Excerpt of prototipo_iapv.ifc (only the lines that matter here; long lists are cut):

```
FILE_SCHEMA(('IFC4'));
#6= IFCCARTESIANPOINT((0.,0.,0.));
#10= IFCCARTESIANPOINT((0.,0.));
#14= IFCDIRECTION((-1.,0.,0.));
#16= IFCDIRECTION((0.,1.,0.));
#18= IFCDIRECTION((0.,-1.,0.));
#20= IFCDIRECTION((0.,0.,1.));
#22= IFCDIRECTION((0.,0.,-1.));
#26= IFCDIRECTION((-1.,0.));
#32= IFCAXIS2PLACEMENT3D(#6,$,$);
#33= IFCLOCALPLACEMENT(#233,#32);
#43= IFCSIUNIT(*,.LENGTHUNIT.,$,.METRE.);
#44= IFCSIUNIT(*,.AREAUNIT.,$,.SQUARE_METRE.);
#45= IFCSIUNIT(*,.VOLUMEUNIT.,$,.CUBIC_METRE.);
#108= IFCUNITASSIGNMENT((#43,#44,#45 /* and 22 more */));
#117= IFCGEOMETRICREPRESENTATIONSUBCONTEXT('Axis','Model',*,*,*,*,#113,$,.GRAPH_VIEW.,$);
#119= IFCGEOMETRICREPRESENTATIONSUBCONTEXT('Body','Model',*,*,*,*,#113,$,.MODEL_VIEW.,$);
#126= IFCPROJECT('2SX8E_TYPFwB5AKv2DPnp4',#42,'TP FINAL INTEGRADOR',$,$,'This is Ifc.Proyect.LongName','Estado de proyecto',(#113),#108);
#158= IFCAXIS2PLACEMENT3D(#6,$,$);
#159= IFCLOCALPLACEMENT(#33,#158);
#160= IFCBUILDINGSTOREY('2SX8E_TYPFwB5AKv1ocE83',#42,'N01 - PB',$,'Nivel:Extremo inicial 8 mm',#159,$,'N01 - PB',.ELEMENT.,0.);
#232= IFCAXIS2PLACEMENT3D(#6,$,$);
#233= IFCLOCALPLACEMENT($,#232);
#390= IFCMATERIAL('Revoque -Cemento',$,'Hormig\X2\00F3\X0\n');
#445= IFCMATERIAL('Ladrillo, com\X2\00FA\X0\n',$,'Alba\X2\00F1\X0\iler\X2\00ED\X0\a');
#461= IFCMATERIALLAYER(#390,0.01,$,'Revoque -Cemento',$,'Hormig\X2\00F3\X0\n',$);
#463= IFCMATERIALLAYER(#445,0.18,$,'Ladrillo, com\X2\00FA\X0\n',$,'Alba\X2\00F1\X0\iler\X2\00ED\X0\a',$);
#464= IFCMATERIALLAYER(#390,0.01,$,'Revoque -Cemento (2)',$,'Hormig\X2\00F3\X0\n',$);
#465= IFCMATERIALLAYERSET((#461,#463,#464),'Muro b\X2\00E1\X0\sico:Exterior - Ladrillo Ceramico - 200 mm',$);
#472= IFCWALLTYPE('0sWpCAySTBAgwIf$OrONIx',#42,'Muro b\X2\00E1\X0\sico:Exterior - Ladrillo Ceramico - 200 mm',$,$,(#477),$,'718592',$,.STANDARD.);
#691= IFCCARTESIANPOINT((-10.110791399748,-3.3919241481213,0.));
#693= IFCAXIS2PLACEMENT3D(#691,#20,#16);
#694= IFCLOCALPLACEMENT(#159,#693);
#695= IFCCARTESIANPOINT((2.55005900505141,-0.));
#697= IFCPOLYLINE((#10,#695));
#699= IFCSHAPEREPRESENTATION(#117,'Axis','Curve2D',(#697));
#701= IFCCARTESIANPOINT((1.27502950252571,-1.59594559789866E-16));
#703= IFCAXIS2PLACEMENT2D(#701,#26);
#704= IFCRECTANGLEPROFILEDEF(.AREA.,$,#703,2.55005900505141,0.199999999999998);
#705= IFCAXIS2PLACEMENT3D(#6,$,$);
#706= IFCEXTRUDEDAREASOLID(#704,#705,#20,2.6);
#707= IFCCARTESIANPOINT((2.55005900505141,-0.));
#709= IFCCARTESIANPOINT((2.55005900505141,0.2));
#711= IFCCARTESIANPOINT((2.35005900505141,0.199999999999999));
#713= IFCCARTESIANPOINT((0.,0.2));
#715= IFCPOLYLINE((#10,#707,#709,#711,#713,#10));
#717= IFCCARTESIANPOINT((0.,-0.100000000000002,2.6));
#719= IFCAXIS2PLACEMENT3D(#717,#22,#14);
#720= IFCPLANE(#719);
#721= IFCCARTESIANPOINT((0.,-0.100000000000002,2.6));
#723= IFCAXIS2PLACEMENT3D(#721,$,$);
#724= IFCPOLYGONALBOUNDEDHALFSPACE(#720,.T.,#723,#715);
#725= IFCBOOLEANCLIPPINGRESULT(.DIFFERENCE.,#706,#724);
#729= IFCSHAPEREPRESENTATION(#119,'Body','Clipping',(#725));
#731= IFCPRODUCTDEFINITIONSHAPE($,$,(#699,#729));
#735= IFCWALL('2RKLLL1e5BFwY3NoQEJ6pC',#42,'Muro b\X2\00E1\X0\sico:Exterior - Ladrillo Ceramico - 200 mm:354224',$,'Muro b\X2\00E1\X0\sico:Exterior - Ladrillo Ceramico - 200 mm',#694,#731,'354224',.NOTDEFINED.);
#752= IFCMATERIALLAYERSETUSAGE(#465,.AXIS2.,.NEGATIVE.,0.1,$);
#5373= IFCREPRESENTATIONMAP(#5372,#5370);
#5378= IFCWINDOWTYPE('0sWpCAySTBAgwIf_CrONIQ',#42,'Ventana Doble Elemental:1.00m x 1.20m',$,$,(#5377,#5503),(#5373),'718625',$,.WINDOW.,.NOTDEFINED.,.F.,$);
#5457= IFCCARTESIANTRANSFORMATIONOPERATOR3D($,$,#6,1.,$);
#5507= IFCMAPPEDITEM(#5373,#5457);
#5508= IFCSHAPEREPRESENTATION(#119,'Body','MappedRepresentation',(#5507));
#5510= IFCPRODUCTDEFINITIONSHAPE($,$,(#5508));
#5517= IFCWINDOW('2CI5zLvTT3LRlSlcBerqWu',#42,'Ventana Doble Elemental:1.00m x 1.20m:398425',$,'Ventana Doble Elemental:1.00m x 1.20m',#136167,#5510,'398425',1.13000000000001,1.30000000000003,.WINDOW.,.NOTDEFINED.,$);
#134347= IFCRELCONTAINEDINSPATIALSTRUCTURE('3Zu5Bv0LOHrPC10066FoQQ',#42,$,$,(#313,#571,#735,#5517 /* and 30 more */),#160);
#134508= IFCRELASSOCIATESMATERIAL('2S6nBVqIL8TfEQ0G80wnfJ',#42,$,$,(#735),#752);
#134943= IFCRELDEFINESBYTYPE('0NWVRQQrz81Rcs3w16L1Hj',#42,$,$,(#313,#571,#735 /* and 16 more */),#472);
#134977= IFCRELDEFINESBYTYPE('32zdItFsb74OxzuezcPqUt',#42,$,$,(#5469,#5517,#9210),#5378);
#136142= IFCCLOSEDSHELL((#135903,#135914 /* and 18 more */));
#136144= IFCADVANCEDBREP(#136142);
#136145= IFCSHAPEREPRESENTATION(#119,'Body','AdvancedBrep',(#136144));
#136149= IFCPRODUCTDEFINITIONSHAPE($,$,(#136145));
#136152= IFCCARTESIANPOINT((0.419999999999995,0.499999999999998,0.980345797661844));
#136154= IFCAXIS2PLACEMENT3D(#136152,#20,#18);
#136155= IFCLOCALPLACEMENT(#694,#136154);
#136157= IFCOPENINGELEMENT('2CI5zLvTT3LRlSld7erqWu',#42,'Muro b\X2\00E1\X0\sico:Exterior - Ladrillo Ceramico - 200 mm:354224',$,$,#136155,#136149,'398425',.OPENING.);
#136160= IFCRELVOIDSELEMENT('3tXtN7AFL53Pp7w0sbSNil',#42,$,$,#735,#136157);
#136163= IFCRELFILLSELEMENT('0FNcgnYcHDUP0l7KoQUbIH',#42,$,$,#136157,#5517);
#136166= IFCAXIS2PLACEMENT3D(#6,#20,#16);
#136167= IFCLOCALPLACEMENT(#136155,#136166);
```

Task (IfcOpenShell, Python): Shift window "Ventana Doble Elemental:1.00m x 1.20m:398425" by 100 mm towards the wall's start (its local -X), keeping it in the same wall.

```python
import ifcopenshell
import ifcopenshell.api.geometry
import ifcopenshell.util.placement
import ifcopenshell.util.unit

model = ifcopenshell.open("prototipo_iapv.ifc")
unit_scale = ifcopenshell.util.unit.calculate_unit_scale(model)

window = model.by_guid("2CI5zLvTT3LRlSlcBerqWu")
opening = window.FillsVoids[0].RelatingOpeningElement
wall = opening.VoidsElements[0].RelatingBuildingElement

wall_matrix = ifcopenshell.util.placement.get_local_placement(wall.ObjectPlacement)
shift = wall_matrix[:3, 0] * -0.1 / unit_scale
before = ifcopenshell.util.placement.get_local_placement(window.ObjectPlacement)[:3, 3].copy()

# The window is placed relative to its opening, so it follows when the opening moves.
matrix = ifcopenshell.util.placement.get_local_placement(opening.ObjectPlacement)
matrix[:3, 3] += shift
ifcopenshell.api.geometry.edit_object_placement(
    model, product=opening, matrix=matrix, is_si=False, should_transform_children=True
)

after = ifcopenshell.util.placement.get_local_placement(window.ObjectPlacement)[:3, 3]
print("window moved by", (after - before).round(3) + 0.0)

model.write("prototipo_iapv_updated.ifc")
```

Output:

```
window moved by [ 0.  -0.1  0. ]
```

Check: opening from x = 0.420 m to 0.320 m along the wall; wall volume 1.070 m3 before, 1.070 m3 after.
